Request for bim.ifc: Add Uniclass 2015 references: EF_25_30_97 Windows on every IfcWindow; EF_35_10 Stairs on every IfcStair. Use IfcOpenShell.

First a look at what the model holds.

```python
import ifcopenshell

model = ifcopenshell.open("bim.ifc")
print(model.schema)
print("classifications:", [c.Name for c in model.by_type("IfcClassification")])
for ifc_class in ("IfcDoor", "IfcRoof", "IfcStair", "IfcWall", "IfcWindow"):
    print(ifc_class, len(model.by_type(ifc_class)))
```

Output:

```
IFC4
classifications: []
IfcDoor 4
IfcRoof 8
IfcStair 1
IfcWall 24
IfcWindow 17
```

```python
import ifcopenshell
import ifcopenshell.api.classification

model = ifcopenshell.open("bim.ifc")

system = ifcopenshell.api.classification.add_classification(model, classification="Uniclass 2015")

codes = {
    "IfcWindow": ("EF_25_30_97", "Windows"),
    "IfcStair": ("EF_35_10", "Stairs"),
}
for ifc_class, (code, name) in codes.items():
    products = model.by_type(ifc_class)
    ifcopenshell.api.classification.add_reference(
        model, products=products, classification=system, identification=code, name=name
    )
    print(code, len(products))

model.write("bim_v2.ifc")
```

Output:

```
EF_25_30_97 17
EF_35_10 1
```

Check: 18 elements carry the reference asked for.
